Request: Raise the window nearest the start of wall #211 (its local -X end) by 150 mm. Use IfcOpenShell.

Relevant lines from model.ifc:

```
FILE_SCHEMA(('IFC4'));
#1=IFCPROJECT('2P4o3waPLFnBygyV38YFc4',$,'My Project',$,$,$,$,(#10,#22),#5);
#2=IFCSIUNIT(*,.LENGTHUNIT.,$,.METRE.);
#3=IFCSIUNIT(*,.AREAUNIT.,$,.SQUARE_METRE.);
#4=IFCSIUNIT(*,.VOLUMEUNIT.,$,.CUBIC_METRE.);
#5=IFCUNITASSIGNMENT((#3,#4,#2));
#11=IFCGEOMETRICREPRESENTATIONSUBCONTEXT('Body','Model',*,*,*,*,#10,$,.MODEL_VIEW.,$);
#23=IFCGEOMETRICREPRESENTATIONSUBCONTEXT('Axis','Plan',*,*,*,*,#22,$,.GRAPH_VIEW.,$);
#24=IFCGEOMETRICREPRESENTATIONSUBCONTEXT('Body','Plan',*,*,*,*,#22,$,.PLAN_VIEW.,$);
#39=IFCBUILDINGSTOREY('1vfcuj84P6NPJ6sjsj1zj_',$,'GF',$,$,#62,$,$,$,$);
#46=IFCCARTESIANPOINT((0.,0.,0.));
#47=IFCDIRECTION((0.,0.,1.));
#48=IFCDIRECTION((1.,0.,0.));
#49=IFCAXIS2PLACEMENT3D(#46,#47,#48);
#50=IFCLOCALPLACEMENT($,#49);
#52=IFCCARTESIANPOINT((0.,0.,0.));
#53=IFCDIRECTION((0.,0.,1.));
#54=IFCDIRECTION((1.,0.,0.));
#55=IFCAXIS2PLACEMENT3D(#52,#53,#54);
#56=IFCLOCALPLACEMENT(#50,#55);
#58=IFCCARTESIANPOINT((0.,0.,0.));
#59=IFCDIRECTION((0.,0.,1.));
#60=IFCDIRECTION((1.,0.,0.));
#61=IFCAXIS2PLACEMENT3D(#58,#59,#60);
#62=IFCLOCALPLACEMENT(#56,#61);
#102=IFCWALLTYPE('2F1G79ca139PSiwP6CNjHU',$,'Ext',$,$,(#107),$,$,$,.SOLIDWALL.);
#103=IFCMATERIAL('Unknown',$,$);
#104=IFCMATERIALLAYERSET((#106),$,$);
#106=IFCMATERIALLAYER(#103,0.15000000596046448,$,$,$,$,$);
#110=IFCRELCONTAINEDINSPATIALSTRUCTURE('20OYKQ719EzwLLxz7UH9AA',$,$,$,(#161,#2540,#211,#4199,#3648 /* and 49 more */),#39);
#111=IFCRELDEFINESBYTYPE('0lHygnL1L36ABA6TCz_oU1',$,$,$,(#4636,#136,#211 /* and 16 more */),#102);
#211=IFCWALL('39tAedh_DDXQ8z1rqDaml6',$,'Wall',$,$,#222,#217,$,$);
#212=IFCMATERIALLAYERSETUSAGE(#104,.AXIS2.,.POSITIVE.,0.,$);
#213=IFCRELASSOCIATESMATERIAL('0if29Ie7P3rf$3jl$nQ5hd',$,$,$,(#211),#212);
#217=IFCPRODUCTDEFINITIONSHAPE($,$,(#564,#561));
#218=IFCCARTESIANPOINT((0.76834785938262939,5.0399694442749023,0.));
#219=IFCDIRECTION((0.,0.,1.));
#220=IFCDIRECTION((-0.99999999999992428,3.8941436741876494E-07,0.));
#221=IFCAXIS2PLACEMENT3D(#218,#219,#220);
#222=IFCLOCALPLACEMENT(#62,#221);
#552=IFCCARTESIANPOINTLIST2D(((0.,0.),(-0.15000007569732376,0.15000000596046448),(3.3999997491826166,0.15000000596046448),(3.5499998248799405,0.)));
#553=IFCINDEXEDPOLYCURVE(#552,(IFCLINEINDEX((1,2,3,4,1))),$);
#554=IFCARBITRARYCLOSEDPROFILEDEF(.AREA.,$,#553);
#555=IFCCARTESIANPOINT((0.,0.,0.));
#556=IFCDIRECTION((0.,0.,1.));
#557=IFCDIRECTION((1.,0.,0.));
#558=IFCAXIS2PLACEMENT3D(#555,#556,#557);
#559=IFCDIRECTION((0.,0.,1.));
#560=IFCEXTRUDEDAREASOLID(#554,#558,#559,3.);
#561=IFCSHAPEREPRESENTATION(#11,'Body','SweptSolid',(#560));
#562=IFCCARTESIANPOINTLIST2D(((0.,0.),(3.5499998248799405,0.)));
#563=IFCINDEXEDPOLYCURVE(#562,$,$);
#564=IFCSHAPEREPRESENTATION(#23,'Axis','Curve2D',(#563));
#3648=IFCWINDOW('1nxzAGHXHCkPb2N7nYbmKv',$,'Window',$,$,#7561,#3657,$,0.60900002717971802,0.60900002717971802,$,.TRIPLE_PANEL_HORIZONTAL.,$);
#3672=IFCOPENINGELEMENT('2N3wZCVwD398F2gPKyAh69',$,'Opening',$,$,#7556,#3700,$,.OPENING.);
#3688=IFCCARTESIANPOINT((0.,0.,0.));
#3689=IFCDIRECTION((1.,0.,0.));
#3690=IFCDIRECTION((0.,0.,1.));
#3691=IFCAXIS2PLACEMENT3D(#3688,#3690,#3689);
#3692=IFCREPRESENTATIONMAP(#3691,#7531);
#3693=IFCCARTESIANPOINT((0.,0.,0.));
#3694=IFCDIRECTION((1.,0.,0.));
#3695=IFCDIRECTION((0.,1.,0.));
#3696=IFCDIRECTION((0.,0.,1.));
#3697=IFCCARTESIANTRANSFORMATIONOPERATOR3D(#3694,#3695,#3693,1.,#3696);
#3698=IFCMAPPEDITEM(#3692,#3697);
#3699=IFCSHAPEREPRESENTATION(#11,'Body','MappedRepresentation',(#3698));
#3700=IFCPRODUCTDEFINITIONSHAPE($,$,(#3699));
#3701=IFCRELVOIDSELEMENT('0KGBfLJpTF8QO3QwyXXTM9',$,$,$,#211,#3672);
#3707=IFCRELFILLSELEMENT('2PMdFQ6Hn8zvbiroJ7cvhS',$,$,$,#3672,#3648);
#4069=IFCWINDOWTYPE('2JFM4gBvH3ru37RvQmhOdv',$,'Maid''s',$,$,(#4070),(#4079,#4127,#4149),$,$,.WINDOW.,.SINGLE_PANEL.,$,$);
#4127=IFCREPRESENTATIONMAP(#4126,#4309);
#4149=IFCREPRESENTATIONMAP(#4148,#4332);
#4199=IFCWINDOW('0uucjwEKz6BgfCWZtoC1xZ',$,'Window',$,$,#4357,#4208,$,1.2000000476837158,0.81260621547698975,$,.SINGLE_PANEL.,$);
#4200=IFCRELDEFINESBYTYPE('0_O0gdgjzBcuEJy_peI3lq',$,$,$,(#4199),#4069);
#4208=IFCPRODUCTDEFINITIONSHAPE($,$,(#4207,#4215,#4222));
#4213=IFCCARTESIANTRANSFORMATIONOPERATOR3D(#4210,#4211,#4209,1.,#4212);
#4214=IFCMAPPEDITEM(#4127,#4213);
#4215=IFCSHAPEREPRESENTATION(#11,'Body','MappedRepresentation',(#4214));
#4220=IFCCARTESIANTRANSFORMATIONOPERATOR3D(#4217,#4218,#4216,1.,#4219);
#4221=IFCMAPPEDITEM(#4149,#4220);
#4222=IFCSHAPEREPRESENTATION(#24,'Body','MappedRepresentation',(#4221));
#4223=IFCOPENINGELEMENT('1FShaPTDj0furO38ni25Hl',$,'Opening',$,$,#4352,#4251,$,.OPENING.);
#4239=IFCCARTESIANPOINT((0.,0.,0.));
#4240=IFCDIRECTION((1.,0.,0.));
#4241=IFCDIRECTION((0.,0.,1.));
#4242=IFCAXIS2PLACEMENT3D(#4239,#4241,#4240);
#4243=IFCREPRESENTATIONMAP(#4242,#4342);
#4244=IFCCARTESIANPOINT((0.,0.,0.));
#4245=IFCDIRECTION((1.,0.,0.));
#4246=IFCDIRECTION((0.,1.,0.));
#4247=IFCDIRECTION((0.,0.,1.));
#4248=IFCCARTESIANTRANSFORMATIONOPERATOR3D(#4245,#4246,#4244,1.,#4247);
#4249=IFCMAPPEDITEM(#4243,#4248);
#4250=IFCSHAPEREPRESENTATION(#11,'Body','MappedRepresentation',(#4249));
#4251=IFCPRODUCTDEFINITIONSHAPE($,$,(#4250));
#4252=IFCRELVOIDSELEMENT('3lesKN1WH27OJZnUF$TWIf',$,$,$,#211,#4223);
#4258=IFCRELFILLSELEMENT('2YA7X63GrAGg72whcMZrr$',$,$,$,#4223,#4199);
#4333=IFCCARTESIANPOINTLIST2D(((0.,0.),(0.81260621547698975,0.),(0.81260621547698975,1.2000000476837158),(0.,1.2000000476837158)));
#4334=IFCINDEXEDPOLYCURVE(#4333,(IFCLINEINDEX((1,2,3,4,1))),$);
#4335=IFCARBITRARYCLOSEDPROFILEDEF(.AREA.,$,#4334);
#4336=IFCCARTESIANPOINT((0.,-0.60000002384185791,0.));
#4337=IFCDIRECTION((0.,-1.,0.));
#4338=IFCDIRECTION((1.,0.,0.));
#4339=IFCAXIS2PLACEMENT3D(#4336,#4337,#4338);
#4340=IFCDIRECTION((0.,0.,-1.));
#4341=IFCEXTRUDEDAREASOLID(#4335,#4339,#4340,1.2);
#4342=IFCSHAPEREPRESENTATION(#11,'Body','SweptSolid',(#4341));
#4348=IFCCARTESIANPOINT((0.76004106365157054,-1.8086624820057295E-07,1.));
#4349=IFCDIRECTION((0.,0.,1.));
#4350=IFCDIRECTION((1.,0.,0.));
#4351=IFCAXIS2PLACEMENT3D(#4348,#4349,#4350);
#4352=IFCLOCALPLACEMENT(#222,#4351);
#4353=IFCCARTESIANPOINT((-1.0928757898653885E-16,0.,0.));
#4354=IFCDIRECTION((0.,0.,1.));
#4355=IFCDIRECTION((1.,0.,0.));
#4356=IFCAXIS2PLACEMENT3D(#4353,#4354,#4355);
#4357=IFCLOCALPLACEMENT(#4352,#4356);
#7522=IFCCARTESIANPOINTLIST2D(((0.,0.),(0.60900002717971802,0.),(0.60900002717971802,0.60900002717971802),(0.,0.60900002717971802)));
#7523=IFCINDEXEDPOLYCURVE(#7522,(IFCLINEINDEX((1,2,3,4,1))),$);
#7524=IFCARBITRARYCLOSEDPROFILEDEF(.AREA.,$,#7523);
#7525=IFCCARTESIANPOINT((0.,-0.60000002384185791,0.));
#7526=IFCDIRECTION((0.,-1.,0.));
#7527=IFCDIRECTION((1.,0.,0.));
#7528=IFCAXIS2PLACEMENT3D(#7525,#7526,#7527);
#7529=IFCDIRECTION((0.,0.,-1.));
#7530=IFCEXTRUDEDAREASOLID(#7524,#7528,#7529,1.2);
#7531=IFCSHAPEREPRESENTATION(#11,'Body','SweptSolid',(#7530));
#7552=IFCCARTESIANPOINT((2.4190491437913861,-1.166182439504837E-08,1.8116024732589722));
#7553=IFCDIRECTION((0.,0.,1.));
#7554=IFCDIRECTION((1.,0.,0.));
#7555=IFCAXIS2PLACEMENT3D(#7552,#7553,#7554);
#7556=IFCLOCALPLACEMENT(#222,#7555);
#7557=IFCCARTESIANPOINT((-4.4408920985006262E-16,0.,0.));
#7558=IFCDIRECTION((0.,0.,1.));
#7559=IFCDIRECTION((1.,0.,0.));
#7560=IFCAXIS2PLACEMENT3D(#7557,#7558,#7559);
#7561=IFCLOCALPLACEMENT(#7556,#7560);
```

```python
import numpy as np
import ifcopenshell
import ifcopenshell.api.geometry
import ifcopenshell.util.placement
import ifcopenshell.util.unit

model = ifcopenshell.open("model.ifc")
unit_scale = ifcopenshell.util.unit.calculate_unit_scale(model)

window = model.by_guid("0uucjwEKz6BgfCWZtoC1xZ")
opening = window.FillsVoids[0].RelatingOpeningElement
dz = 0.15 / unit_scale

shift = np.array([0.0, 0.0, dz])
# The window is placed relative to its opening, so it follows when the opening moves.
matrix = ifcopenshell.util.placement.get_local_placement(opening.ObjectPlacement)
matrix[:3, 3] += shift
ifcopenshell.api.geometry.edit_object_placement(
    model, product=opening, matrix=matrix, is_si=False, should_transform_children=True
)

print(f"moved by {dz * unit_scale:+.3f} m")

model.write("model_rev.ifc")
```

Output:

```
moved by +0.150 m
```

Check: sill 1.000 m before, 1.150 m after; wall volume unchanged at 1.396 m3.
